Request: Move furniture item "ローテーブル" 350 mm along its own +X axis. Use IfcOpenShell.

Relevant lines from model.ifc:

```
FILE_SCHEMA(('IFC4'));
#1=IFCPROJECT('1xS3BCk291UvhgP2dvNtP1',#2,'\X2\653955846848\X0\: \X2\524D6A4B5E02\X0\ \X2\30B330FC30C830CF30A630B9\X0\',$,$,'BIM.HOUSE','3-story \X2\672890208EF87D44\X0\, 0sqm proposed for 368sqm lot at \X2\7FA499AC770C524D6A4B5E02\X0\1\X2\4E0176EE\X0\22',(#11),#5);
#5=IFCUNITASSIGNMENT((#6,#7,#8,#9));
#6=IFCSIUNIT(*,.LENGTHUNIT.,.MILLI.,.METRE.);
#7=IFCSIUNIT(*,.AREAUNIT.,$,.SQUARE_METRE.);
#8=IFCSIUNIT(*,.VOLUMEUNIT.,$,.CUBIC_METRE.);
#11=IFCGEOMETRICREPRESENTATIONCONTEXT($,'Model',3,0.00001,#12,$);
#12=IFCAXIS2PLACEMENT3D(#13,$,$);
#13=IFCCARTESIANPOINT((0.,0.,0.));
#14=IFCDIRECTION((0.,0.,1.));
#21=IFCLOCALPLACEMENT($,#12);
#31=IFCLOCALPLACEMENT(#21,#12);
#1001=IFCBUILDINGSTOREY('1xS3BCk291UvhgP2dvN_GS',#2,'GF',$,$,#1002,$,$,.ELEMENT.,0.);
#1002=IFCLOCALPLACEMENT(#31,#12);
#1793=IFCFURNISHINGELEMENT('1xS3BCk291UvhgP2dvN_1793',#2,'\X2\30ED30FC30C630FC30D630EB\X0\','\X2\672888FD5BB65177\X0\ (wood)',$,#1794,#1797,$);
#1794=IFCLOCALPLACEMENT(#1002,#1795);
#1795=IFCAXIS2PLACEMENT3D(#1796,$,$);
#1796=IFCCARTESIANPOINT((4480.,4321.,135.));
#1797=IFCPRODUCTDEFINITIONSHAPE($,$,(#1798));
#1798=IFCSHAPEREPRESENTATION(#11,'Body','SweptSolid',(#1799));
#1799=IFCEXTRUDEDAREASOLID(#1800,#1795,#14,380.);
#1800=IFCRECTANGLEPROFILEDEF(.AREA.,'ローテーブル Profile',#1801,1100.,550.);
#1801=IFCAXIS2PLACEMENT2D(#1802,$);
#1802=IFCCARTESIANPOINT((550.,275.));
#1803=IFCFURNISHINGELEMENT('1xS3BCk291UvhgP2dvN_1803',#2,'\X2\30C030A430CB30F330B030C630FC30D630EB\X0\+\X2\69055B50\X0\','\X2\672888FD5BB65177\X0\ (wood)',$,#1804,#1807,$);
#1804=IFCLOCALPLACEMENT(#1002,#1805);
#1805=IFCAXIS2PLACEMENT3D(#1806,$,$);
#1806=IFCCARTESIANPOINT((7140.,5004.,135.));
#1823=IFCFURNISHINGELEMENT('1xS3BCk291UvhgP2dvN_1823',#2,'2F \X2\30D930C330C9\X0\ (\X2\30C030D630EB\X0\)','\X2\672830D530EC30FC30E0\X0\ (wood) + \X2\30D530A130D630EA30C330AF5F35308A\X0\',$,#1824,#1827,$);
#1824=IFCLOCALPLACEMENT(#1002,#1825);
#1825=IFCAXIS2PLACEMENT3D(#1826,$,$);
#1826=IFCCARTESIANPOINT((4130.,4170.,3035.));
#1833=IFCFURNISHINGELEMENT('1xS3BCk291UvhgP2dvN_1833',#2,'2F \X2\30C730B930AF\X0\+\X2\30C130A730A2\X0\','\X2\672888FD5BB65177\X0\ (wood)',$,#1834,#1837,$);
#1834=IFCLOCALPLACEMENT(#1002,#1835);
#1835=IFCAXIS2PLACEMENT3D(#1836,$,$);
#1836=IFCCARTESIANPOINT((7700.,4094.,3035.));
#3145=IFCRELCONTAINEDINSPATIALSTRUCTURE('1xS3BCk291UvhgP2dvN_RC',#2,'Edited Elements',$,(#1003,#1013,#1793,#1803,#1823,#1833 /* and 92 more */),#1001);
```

```python
import ifcopenshell
import ifcopenshell.api.geometry
import ifcopenshell.util.placement
import ifcopenshell.util.unit

model = ifcopenshell.open("model.ifc")
unit_scale = ifcopenshell.util.unit.calculate_unit_scale(model)

item = model.by_guid("1xS3BCk291UvhgP2dvN_1793")
matrix = ifcopenshell.util.placement.get_local_placement(item.ObjectPlacement)
matrix[:3, 3] += matrix[:3, 0] * 0.35 / unit_scale
ifcopenshell.api.geometry.edit_object_placement(model, product=item, matrix=matrix, is_si=False)

print(ifcopenshell.util.placement.get_local_placement(item.ObjectPlacement).round(3) + 0.0)

model.write("model-out.ifc")
```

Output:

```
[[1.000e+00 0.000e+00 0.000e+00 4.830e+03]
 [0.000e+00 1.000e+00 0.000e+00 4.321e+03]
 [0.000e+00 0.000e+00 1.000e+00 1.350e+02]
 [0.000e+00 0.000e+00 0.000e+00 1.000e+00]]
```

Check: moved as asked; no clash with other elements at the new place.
